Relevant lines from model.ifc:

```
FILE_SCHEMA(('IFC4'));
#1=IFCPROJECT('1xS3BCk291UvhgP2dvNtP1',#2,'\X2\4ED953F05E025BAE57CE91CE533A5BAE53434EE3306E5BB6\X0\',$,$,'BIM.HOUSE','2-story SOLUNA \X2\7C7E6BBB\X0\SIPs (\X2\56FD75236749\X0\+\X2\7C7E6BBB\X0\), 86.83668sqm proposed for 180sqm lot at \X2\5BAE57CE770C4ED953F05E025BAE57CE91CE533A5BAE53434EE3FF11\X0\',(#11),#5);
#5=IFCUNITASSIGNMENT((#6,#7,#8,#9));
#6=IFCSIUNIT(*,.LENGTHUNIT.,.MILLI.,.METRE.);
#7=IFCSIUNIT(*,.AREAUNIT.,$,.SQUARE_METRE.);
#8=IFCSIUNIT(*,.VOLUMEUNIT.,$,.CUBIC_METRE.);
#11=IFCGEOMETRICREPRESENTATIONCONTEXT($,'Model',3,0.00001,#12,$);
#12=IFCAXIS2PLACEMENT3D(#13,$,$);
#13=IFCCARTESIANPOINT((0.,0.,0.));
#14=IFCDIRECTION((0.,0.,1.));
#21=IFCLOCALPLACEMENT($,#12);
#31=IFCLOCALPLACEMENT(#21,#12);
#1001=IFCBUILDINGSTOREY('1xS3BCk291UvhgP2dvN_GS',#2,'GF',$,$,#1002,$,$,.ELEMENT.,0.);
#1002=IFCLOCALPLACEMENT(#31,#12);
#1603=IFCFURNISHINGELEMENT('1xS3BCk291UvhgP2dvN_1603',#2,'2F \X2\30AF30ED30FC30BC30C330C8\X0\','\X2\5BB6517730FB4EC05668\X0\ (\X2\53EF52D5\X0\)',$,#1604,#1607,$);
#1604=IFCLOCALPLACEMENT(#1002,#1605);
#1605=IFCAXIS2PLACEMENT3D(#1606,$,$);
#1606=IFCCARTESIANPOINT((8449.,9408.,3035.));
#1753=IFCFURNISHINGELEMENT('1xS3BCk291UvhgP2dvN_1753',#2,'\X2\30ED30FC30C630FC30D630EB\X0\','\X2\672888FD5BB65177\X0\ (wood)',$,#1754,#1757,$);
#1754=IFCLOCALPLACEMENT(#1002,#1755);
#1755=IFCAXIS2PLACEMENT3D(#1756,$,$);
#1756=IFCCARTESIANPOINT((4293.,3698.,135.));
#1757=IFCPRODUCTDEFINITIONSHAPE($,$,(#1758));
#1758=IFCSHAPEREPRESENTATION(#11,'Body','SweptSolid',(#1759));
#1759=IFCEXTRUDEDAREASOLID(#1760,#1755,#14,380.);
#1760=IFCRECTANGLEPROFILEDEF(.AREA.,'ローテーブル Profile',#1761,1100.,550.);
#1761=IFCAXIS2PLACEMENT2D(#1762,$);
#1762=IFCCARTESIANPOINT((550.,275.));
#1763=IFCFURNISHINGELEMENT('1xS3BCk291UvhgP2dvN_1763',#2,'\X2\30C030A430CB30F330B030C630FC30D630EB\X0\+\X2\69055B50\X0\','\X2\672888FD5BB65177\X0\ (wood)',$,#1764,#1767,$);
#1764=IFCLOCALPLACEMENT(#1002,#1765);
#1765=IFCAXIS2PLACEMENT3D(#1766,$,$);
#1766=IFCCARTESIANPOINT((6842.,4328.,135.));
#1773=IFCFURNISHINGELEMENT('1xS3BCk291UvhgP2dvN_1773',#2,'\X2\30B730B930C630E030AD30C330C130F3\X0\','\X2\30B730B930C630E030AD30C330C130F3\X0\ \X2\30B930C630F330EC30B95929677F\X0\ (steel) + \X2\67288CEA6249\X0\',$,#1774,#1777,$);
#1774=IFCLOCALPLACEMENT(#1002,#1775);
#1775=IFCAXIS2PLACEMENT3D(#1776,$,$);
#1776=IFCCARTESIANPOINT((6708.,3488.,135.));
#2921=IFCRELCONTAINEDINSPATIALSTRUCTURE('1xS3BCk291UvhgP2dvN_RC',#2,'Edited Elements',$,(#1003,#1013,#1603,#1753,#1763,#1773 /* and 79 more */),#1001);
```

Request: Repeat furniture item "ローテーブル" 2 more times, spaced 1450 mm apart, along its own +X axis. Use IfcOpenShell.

```python
import ifcopenshell
import ifcopenshell.api.geometry
import ifcopenshell.api.root
import ifcopenshell.util.element
import ifcopenshell.util.placement

model = ifcopenshell.open("model.ifc")


def reuse_history(source, copy):
    """copy_class also copies each property set's owner history, people and application; keep the originals."""
    for rel in copy.IsDefinedBy:
        if rel.is_a("IfcRelDefinesByProperties") and (history := rel.RelatingPropertyDefinition.OwnerHistory):
            rel.RelatingPropertyDefinition.OwnerHistory = source.OwnerHistory
            ifcopenshell.util.element.remove_deep2(model, history)


source = model.by_id(1753)
base = ifcopenshell.util.placement.get_local_placement(source.ObjectPlacement)
step = base[:3, 0] * 1450.0

for i in range(1, 3):
    copy = ifcopenshell.api.root.copy_class(model, product=source)
    copy.Representation = ifcopenshell.util.element.copy_deep(
        model, source.Representation, exclude=["IfcGeometricRepresentationContext", "IfcRepresentationMap"]
    )
    reuse_history(source, copy)
    matrix = base.copy()
    matrix[:3, 3] += i * step
    print("added at", matrix[:3, 3].round(3) + 0.0)
    ifcopenshell.api.geometry.edit_object_placement(model, product=copy, matrix=matrix, is_si=False)

model.write("model_v2.ifc")
```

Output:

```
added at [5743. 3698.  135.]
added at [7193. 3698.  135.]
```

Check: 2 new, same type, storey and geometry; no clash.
